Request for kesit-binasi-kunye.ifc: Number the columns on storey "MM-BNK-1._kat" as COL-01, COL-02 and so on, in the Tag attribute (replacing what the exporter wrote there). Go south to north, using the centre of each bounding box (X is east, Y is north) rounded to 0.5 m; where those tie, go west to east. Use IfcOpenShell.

First a look at what the model holds.

```python
import ifcopenshell
import ifcopenshell.util.element
import ifcopenshell.util.placement

model = ifcopenshell.open("kesit-binasi-kunye.ifc")
print(model.schema)
storey = next(s for s in model.by_type("IfcBuildingStorey") if s.Name == "MM-BNK-1._kat")
columns = [e for e in ifcopenshell.util.element.get_decomposition(storey) if e.is_a("IfcColumn")]
for e in sorted(columns, key=lambda e: e.id()):
    origin = ifcopenshell.util.placement.get_local_placement(e.ObjectPlacement)[:3, 3]
    print(e.id(), e.Tag, e.Name, origin.round(2) + 0.0, sep=" | ")
```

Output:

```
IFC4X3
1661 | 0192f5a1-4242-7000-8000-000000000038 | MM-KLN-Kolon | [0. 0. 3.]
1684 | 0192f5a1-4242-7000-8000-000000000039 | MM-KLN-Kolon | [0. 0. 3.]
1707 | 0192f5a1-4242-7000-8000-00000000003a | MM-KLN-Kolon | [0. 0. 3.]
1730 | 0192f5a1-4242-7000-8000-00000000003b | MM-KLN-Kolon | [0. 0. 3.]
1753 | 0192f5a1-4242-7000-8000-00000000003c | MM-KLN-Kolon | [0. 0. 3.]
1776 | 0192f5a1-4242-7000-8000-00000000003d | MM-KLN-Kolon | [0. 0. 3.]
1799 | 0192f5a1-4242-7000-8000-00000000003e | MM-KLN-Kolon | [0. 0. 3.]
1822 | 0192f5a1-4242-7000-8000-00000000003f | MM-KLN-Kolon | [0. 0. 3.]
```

```python
import ifcopenshell
import ifcopenshell.geom
import ifcopenshell.util.element
import ifcopenshell.util.shape

model = ifcopenshell.open("kesit-binasi-kunye.ifc")
settings = ifcopenshell.geom.settings()
settings.set("use-world-coords", True)


def centre(element):
    shape = ifcopenshell.geom.create_shape(settings, element)
    return ifcopenshell.util.shape.get_bbox_centroid(shape.geometry)


storey = next(s for s in model.by_type("IfcBuildingStorey") if s.Name == "MM-BNK-1._kat")
columns = [e for e in ifcopenshell.util.element.get_decomposition(storey) if e.is_a("IfcColumn")]

# Insertion points can sit at a corner or the storey origin, so sort by the geometry (in metres).
centres = {e: centre(e) for e in columns}
columns.sort(key=lambda e: (round(centres[e][1] / 0.5), centres[e][0]))

for i, e in enumerate(columns, start=1):
    number = f"COL-{i:02d}"
    e.Tag = number
    print(e.id(), number)

model.write("kesit-binasi-kunye_updated.ifc")
```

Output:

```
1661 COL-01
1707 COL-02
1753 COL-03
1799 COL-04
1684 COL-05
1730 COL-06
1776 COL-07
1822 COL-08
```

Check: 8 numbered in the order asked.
